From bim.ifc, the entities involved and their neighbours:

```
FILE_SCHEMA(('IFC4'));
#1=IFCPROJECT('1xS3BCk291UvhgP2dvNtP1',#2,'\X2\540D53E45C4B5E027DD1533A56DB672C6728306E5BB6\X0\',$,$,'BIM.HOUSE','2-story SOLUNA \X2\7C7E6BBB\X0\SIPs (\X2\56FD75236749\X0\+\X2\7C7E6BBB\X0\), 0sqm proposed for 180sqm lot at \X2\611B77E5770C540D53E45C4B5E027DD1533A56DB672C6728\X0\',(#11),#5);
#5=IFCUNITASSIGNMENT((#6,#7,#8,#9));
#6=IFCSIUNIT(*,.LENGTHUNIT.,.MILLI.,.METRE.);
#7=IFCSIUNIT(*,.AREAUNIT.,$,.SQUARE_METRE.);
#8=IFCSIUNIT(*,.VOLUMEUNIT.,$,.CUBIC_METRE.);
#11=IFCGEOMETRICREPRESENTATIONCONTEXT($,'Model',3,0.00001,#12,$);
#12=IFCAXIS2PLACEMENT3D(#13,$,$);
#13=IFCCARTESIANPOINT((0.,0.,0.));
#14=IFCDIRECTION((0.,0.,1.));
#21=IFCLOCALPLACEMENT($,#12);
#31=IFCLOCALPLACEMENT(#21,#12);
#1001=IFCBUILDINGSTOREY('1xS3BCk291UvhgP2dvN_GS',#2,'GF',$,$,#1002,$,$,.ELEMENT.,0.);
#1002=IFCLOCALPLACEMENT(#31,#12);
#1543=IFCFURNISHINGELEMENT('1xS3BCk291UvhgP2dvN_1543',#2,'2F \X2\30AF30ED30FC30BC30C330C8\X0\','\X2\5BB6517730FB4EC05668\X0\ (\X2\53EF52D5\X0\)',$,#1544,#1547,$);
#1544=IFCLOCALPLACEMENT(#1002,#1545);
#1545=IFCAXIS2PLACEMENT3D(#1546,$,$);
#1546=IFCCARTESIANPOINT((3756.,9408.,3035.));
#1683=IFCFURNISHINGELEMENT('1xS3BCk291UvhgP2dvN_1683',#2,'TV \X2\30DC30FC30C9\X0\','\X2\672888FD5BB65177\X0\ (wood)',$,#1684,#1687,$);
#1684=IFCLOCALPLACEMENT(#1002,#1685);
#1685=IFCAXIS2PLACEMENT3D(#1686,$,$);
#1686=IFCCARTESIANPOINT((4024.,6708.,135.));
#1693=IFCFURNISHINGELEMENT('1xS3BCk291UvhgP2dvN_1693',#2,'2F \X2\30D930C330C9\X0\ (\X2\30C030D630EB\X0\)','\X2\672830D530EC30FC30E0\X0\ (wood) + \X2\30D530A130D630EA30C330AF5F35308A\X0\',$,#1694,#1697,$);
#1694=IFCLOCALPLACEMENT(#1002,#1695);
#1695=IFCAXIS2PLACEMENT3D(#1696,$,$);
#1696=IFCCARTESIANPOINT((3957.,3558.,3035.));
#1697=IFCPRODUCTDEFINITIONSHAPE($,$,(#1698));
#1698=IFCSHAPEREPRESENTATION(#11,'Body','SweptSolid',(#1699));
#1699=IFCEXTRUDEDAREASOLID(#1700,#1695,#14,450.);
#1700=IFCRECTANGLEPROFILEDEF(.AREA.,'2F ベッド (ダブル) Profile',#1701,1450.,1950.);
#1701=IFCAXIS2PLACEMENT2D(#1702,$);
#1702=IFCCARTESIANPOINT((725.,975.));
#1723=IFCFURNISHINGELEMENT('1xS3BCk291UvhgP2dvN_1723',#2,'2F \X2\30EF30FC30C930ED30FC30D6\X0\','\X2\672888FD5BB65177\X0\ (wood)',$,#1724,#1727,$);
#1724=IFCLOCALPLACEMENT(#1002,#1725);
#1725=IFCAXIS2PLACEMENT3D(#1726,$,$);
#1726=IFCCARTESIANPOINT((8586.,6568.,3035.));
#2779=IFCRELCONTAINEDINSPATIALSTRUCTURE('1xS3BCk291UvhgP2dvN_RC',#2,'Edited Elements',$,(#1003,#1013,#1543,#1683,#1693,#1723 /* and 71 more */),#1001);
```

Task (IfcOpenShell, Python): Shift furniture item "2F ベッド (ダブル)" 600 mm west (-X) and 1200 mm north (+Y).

```python
import ifcopenshell
import ifcopenshell.api.geometry
import ifcopenshell.util.placement
import ifcopenshell.util.unit

model = ifcopenshell.open("bim.ifc")
unit_scale = ifcopenshell.util.unit.calculate_unit_scale(model)

item = model.by_guid("1xS3BCk291UvhgP2dvN_1693")
matrix = ifcopenshell.util.placement.get_local_placement(item.ObjectPlacement)
matrix[0, 3] -= 0.6 / unit_scale
matrix[1, 3] += 1.2 / unit_scale
ifcopenshell.api.geometry.edit_object_placement(model, product=item, matrix=matrix, is_si=False)

print(ifcopenshell.util.placement.get_local_placement(item.ObjectPlacement).round(3) + 0.0)

model.write("bim-out.ifc")
```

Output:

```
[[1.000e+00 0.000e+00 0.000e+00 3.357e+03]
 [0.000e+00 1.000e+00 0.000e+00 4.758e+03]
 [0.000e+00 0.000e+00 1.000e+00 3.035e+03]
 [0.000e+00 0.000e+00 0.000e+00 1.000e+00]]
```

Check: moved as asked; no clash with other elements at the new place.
